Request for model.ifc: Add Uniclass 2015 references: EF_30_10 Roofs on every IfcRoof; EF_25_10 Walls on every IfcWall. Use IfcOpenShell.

First a look at what the model holds.

```python
import ifcopenshell

model = ifcopenshell.open("model.ifc")
print(model.schema)
print("classifications:", [c.Name for c in model.by_type("IfcClassification")])
for ifc_class in ("IfcDoor", "IfcRoof", "IfcStair", "IfcWall", "IfcWindow"):
    print(ifc_class, len(model.by_type(ifc_class)))
```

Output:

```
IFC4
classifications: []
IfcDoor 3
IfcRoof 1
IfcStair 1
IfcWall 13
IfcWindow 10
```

```python
import ifcopenshell
import ifcopenshell.api.classification

model = ifcopenshell.open("model.ifc")

system = ifcopenshell.api.classification.add_classification(model, classification="Uniclass 2015")

codes = {
    "IfcRoof": ("EF_30_10", "Roofs"),
    "IfcWall": ("EF_25_10", "Walls"),
}
for ifc_class, (code, name) in codes.items():
    products = model.by_type(ifc_class)
    ifcopenshell.api.classification.add_reference(
        model, products=products, classification=system, identification=code, name=name
    )
    print(code, len(products))

model.write("model_edited.ifc")
```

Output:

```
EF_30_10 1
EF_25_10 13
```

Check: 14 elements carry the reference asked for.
